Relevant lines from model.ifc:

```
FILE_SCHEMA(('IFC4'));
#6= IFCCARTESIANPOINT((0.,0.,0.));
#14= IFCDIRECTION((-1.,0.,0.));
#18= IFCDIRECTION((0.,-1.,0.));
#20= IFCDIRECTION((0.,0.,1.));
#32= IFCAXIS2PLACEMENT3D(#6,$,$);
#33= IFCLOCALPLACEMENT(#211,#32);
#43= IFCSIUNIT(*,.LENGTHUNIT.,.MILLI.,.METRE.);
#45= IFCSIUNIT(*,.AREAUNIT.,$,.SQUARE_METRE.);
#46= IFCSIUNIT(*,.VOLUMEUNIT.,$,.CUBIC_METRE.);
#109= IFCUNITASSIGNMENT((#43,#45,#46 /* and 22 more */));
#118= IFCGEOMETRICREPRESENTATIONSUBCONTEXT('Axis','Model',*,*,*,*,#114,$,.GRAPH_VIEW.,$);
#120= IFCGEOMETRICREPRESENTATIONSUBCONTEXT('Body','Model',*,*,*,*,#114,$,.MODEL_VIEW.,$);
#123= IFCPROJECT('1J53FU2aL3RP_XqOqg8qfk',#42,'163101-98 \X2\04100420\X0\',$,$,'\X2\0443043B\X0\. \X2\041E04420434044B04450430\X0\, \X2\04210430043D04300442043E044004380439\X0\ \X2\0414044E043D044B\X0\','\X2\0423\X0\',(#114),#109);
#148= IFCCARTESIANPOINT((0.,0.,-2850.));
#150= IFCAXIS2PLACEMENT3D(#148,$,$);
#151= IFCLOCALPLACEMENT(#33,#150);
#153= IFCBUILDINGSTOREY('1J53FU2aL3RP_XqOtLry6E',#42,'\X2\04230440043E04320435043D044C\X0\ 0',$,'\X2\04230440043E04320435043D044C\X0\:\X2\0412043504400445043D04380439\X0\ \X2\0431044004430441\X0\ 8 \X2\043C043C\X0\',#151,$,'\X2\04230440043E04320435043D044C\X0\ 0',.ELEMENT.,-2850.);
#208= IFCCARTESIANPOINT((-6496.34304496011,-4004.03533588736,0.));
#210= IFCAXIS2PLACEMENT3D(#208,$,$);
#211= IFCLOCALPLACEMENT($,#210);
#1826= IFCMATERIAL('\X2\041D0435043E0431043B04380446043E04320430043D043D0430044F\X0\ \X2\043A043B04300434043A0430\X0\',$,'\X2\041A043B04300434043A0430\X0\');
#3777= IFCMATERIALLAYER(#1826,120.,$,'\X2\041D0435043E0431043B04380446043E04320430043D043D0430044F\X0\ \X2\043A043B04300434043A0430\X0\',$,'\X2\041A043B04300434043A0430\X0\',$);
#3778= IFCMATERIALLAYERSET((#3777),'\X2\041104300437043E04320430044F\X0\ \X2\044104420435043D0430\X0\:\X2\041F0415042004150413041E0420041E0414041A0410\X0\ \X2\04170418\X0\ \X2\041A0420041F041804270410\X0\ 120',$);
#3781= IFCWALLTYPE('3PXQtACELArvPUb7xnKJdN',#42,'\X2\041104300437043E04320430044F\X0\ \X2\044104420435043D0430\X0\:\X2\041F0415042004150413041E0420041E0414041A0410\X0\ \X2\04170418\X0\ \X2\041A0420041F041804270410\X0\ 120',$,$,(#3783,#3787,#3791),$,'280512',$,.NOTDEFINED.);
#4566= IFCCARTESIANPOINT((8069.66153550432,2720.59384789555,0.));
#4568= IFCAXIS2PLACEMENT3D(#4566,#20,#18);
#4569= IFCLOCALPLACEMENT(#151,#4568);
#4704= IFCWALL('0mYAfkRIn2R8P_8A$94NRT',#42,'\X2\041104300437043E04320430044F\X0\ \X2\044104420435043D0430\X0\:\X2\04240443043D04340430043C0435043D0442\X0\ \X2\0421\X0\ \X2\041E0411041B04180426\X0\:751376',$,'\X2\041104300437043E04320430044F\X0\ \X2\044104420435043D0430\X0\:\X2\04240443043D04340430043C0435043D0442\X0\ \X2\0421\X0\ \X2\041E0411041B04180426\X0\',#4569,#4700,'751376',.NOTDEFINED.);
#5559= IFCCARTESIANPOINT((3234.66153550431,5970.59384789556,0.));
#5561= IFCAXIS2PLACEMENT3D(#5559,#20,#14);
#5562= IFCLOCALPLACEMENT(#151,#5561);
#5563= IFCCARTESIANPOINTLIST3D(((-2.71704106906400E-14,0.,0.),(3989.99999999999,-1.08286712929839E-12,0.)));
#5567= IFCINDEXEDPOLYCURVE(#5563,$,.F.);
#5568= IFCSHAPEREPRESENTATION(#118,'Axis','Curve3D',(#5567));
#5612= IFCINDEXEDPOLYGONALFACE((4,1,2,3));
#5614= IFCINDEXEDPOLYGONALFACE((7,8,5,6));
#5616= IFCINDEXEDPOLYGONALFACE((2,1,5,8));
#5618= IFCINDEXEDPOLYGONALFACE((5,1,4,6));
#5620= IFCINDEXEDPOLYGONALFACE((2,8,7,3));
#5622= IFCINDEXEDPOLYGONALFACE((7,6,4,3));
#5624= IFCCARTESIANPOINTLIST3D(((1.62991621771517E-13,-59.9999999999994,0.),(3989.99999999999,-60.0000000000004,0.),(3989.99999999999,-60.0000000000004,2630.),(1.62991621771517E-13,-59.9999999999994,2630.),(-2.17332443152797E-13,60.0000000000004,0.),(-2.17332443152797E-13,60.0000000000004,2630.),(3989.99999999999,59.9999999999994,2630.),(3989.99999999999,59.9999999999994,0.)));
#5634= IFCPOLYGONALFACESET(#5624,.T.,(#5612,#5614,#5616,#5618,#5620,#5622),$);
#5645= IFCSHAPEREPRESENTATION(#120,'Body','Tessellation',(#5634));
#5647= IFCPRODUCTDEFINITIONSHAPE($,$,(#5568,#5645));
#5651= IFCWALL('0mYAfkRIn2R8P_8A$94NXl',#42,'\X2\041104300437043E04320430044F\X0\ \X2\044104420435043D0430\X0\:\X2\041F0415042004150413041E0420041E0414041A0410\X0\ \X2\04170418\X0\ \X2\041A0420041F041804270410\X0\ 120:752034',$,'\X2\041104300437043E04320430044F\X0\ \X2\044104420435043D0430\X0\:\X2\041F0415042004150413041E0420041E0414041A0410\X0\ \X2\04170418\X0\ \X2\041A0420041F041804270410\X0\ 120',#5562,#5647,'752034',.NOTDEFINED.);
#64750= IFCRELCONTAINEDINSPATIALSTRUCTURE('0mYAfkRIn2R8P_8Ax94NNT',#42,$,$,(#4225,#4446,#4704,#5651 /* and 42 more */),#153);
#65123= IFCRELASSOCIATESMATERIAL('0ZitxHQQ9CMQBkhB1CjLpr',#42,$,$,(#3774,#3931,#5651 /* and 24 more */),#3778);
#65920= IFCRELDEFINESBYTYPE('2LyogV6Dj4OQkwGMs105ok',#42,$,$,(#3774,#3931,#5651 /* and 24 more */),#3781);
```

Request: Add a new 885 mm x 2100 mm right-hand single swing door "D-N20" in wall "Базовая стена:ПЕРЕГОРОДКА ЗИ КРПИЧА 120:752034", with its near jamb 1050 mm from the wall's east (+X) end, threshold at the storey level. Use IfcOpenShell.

```python
import numpy as np
import ifcopenshell
import ifcopenshell.api.feature
import ifcopenshell.api.geometry
import ifcopenshell.api.root
import ifcopenshell.api.spatial
import ifcopenshell.geom
import ifcopenshell.util.element
import ifcopenshell.util.placement
import ifcopenshell.util.representation
import ifcopenshell.util.shape
import ifcopenshell.util.unit

model = ifcopenshell.open("model.ifc")
unit_scale = ifcopenshell.util.unit.calculate_unit_scale(model)
settings = ifcopenshell.geom.settings()


def volume(element):
    """Net volume in cubic metres, openings subtracted."""
    shape = ifcopenshell.geom.create_shape(settings, element)
    return ifcopenshell.util.shape.get_volume(shape.geometry)


wall = model.by_id(5651)
storey = ifcopenshell.util.element.get_container(wall, ifc_class="IfcBuildingStorey")
context = ifcopenshell.util.representation.get_context(model, "Model", "Body", "MODEL_VIEW")
before = volume(wall)

width, height, from_end, sill = 0.885, 2.1, 1.05, 0.0  # metres

# The wall runs along its own X axis, and the end named is its -X end.
wall_shape = ifcopenshell.geom.create_shape(settings, wall)
x, y, z = ifcopenshell.util.shape.get_vertices(wall_shape.geometry).T
start = x.min() + from_end
face, thickness = float(y.min()), float(y.max() - y.min())
wall_matrix = ifcopenshell.util.placement.get_local_placement(wall.ObjectPlacement)
level = ifcopenshell.util.placement.get_local_placement(storey.ObjectPlacement)[2, 3]


def in_wall(x, y):
    """Placement at x, y metres in the wall's axes, at sill height."""
    matrix = wall_matrix.copy()
    matrix[:, 3] = wall_matrix @ np.array([x / unit_scale, y / unit_scale, 0.0, 1.0])
    matrix[2, 3] = level + sill / unit_scale
    return matrix


# Opening: a box that overshoots both wall faces by 50 mm.
opening = ifcopenshell.api.root.create_entity(model, ifc_class="IfcOpeningElement", predefined_type="OPENING")
box = ifcopenshell.api.geometry.add_wall_representation(
    model, context=context, length=width, height=height, thickness=thickness + 0.1
)
ifcopenshell.api.geometry.assign_representation(model, product=opening, representation=box)
ifcopenshell.api.geometry.edit_object_placement(model, product=opening, matrix=in_wall(start, face - 0.05), is_si=False)
ifcopenshell.api.feature.add_feature(model, feature=opening, element=wall)

door = ifcopenshell.api.root.create_entity(model, ifc_class="IfcDoor", name="D-N20", predefined_type="DOOR")
door.OverallWidth, door.OverallHeight = width / unit_scale, height / unit_scale
door.OperationType = "SINGLE_SWING_RIGHT"
body = ifcopenshell.api.geometry.add_door_representation(
    model,
    context=context,
    overall_width=door.OverallWidth,
    overall_height=door.OverallHeight,
    operation_type="SINGLE_SWING_RIGHT",
    lining_properties={"LiningDepth": thickness / unit_scale, "ThresholdDepth": thickness / unit_scale},
)
ifcopenshell.api.geometry.assign_representation(model, product=door, representation=body)
ifcopenshell.api.spatial.assign_container(model, products=[door], relating_structure=storey)
ifcopenshell.api.feature.add_filling(model, opening=opening, element=door)

# The lining spans the wall, so the door starts at the wall face.
ifcopenshell.api.geometry.edit_object_placement(model, product=door, matrix=in_wall(start, face), is_si=False)

after = volume(wall)

print(f"wall volume {before:.3f} -> {after:.3f} m3")

model.write("model-out.ifc")
```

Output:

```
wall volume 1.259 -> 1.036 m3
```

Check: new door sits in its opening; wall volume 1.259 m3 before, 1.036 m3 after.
